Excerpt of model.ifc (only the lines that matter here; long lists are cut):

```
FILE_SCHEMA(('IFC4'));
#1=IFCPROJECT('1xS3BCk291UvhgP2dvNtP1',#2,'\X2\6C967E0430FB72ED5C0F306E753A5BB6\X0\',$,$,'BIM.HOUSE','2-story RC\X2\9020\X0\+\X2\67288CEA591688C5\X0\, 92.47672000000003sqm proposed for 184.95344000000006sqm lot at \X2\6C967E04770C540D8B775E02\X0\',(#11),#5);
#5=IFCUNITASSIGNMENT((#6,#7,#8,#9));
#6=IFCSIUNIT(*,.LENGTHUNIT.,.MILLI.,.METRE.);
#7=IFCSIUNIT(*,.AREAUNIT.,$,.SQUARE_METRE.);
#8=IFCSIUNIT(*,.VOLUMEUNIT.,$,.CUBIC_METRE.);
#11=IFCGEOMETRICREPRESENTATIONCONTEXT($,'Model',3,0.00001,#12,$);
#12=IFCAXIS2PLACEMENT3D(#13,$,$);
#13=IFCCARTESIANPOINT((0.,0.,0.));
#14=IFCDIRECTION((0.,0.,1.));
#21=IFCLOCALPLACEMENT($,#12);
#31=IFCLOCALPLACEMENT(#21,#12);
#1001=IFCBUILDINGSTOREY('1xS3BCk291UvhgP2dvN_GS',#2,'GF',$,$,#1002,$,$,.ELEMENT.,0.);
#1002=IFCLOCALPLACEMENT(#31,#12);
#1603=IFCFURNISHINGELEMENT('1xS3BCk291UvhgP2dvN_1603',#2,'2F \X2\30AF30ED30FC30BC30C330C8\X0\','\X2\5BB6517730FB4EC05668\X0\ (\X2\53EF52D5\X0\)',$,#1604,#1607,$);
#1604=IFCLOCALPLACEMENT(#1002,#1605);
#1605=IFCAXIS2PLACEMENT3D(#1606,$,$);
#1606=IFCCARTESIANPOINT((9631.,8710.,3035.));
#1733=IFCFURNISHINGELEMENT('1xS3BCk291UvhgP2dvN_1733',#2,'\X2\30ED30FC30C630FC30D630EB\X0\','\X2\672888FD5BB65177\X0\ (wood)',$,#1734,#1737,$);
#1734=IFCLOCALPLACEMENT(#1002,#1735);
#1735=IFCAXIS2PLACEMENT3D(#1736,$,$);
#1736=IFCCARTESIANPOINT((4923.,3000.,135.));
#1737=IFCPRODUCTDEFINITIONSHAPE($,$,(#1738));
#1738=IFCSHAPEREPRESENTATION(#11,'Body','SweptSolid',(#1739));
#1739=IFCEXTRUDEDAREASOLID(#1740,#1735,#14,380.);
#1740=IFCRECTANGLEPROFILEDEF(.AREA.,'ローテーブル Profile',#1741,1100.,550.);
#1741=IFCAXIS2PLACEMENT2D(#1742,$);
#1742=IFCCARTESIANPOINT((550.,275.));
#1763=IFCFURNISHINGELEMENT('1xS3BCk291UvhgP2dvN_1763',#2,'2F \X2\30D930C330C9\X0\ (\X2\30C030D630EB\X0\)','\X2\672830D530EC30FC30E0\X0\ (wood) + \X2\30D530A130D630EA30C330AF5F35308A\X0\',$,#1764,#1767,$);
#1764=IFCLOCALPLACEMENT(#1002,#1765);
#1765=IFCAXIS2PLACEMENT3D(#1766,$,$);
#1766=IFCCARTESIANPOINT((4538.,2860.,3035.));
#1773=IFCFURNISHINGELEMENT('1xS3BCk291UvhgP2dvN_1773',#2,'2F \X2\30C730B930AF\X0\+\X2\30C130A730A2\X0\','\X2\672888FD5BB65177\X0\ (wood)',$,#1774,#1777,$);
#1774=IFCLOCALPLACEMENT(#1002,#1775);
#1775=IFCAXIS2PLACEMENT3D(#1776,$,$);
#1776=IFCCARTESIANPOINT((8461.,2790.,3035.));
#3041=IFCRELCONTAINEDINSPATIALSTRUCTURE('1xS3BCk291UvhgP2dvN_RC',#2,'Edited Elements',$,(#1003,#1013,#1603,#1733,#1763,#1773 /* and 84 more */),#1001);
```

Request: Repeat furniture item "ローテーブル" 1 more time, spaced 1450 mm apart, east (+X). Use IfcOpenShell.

```python
import numpy as np
import ifcopenshell
import ifcopenshell.api.geometry
import ifcopenshell.api.root
import ifcopenshell.util.element
import ifcopenshell.util.placement
import ifcopenshell.util.unit

model = ifcopenshell.open("model.ifc")
unit_scale = ifcopenshell.util.unit.calculate_unit_scale(model)


def reuse_history(source, copy):
    """copy_class also copies each property set's owner history, people and application; keep the originals."""
    for rel in copy.IsDefinedBy:
        if rel.is_a("IfcRelDefinesByProperties") and (history := rel.RelatingPropertyDefinition.OwnerHistory):
            rel.RelatingPropertyDefinition.OwnerHistory = source.OwnerHistory
            ifcopenshell.util.element.remove_deep2(model, history)


source = model.by_guid("1xS3BCk291UvhgP2dvN_1733")
base = ifcopenshell.util.placement.get_local_placement(source.ObjectPlacement)
step = np.array([1.0, 0.0, 0.0]) * 1.45 / unit_scale

for i in range(1, 2):
    copy = ifcopenshell.api.root.copy_class(model, product=source)
    copy.Representation = ifcopenshell.util.element.copy_deep(
        model, source.Representation, exclude=["IfcGeometricRepresentationContext", "IfcRepresentationMap"]
    )
    reuse_history(source, copy)
    matrix = base.copy()
    matrix[:3, 3] += i * step
    print("added at", matrix[:3, 3].round(3) + 0.0)
    ifcopenshell.api.geometry.edit_object_placement(model, product=copy, matrix=matrix, is_si=False)

model.write("model-out.ifc")
```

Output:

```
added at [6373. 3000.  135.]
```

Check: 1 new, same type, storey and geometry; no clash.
